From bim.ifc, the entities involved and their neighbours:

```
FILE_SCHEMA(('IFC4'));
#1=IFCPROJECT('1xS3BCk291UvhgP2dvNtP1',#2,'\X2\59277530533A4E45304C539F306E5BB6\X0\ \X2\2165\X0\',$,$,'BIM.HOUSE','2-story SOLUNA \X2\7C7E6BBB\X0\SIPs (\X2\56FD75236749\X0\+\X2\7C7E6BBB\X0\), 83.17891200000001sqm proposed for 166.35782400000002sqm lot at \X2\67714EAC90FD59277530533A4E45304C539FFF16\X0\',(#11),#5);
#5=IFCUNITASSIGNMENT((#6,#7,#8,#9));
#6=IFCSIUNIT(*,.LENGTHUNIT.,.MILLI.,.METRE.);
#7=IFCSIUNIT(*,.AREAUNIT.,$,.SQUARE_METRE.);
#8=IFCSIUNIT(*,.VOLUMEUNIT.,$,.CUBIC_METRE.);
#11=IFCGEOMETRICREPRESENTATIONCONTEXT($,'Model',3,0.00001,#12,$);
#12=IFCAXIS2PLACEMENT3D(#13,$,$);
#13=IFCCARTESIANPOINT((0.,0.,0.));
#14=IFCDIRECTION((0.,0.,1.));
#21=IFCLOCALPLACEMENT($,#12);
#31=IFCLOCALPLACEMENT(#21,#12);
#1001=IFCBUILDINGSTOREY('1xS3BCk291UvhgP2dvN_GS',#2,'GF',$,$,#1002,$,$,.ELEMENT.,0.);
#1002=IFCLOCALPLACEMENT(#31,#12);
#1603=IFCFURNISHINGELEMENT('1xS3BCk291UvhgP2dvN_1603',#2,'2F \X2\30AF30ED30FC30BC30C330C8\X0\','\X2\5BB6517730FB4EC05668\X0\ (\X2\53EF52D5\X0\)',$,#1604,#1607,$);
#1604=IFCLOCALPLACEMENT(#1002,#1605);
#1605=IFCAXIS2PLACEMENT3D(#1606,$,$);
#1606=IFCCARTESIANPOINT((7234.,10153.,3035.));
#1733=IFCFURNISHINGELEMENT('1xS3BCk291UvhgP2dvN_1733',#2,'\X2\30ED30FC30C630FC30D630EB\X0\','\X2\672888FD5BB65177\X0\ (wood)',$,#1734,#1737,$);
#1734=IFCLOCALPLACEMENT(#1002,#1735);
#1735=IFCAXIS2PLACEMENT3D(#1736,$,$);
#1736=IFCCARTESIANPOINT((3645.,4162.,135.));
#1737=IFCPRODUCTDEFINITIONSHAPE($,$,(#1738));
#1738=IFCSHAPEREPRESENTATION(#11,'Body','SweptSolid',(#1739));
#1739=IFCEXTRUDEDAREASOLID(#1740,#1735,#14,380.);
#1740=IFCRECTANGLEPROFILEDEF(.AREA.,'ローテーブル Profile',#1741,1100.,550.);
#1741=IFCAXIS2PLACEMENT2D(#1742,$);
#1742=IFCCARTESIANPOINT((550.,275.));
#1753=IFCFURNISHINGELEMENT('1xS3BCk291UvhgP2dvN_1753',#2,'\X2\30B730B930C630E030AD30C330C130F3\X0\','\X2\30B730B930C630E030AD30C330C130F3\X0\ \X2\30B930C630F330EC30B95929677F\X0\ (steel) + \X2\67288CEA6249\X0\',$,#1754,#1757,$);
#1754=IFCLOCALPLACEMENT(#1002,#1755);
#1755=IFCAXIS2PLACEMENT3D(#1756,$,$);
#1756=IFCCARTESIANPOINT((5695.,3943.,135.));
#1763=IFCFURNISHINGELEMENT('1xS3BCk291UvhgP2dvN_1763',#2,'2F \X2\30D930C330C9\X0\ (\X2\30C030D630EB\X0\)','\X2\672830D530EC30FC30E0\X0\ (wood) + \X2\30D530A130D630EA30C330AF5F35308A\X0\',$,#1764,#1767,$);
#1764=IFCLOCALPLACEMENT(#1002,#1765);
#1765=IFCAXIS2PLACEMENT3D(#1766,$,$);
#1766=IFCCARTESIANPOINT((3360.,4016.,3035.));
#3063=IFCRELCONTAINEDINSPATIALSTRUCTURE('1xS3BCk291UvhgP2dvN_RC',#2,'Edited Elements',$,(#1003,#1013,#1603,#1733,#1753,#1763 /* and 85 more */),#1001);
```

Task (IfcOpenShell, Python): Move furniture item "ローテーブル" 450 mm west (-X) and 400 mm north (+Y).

```python
import ifcopenshell
import ifcopenshell.api.geometry
import ifcopenshell.util.placement
import ifcopenshell.util.unit

model = ifcopenshell.open("bim.ifc")
unit_scale = ifcopenshell.util.unit.calculate_unit_scale(model)

item = model.by_guid("1xS3BCk291UvhgP2dvN_1733")
matrix = ifcopenshell.util.placement.get_local_placement(item.ObjectPlacement)
matrix[0, 3] -= 0.45 / unit_scale
matrix[1, 3] += 0.4 / unit_scale
ifcopenshell.api.geometry.edit_object_placement(model, product=item, matrix=matrix, is_si=False)

print(ifcopenshell.util.placement.get_local_placement(item.ObjectPlacement).round(3) + 0.0)

model.write("bim-out.ifc")
```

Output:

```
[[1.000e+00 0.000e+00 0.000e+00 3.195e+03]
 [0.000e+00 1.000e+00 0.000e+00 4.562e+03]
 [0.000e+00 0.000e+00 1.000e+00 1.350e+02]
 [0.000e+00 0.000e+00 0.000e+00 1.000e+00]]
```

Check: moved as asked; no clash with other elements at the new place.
